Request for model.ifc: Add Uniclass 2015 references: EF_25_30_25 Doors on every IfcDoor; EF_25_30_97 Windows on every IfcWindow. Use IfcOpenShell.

First a look at what the model holds.

```python
import ifcopenshell

model = ifcopenshell.open("model.ifc")
print(model.schema)
print("classifications:", [c.Name for c in model.by_type("IfcClassification")])
for ifc_class in ("IfcDoor", "IfcRoof", "IfcStair", "IfcWall", "IfcWindow"):
    print(ifc_class, len(model.by_type(ifc_class)))
```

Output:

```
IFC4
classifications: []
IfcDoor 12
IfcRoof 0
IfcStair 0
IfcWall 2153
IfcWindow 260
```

```python
import ifcopenshell
import ifcopenshell.api.classification

model = ifcopenshell.open("model.ifc")

system = ifcopenshell.api.classification.add_classification(model, classification="Uniclass 2015")

codes = {
    "IfcDoor": ("EF_25_30_25", "Doors"),
    "IfcWindow": ("EF_25_30_97", "Windows"),
}
for ifc_class, (code, name) in codes.items():
    products = model.by_type(ifc_class)
    ifcopenshell.api.classification.add_reference(
        model, products=products, classification=system, identification=code, name=name
    )
    print(code, len(products))

model.write("model_edited.ifc")
```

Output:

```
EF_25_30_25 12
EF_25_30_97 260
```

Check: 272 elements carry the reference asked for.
